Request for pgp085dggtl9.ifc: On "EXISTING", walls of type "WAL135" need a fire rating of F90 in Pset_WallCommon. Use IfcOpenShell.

First a look at what the model holds.

```python
import ifcopenshell
import ifcopenshell.util.element

model = ifcopenshell.open("pgp085dggtl9.ifc")
print(model.schema)
storey = next(s for s in model.by_type("IfcBuildingStorey") if s.Name == "EXISTING")
walls = [e for e in ifcopenshell.util.element.get_decomposition(storey) if e.is_a("IfcWall")]
seen = {}
for e in walls:
    element_type = ifcopenshell.util.element.get_type(e)
    key = (element_type.Name if element_type != e and element_type else None, ifcopenshell.util.element.get_pset(e, "Pset_WallCommon", "FireRating"))
    seen[key] = seen.get(key, 0) + 1
for (name, value), count in sorted(seen.items(), key=str):
    print(count, "x", name, "|", value)
```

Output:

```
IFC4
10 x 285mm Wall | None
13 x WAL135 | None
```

```python
import ifcopenshell
import ifcopenshell.api.pset
import ifcopenshell.util.element

model = ifcopenshell.open("pgp085dggtl9.ifc")

storey = next(s for s in model.by_type("IfcBuildingStorey") if s.Name == "EXISTING")
walls = [e for e in ifcopenshell.util.element.get_decomposition(storey) if e.is_a("IfcWall")]

count = 0
for e in walls:
    element_type = ifcopenshell.util.element.get_type(e)
    if element_type in (None, e) or element_type.Name != "WAL135":
        continue
    # add_pset returns the element's existing set when there is one.
    pset = ifcopenshell.api.pset.add_pset(model, product=e, name="Pset_WallCommon")
    ifcopenshell.api.pset.edit_pset(model, pset=pset, properties={"FireRating": "F90"})
    count += 1

print(count, "walls updated")

model.write("pgp085dggtl9_rev.ifc")
```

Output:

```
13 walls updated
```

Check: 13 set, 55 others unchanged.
